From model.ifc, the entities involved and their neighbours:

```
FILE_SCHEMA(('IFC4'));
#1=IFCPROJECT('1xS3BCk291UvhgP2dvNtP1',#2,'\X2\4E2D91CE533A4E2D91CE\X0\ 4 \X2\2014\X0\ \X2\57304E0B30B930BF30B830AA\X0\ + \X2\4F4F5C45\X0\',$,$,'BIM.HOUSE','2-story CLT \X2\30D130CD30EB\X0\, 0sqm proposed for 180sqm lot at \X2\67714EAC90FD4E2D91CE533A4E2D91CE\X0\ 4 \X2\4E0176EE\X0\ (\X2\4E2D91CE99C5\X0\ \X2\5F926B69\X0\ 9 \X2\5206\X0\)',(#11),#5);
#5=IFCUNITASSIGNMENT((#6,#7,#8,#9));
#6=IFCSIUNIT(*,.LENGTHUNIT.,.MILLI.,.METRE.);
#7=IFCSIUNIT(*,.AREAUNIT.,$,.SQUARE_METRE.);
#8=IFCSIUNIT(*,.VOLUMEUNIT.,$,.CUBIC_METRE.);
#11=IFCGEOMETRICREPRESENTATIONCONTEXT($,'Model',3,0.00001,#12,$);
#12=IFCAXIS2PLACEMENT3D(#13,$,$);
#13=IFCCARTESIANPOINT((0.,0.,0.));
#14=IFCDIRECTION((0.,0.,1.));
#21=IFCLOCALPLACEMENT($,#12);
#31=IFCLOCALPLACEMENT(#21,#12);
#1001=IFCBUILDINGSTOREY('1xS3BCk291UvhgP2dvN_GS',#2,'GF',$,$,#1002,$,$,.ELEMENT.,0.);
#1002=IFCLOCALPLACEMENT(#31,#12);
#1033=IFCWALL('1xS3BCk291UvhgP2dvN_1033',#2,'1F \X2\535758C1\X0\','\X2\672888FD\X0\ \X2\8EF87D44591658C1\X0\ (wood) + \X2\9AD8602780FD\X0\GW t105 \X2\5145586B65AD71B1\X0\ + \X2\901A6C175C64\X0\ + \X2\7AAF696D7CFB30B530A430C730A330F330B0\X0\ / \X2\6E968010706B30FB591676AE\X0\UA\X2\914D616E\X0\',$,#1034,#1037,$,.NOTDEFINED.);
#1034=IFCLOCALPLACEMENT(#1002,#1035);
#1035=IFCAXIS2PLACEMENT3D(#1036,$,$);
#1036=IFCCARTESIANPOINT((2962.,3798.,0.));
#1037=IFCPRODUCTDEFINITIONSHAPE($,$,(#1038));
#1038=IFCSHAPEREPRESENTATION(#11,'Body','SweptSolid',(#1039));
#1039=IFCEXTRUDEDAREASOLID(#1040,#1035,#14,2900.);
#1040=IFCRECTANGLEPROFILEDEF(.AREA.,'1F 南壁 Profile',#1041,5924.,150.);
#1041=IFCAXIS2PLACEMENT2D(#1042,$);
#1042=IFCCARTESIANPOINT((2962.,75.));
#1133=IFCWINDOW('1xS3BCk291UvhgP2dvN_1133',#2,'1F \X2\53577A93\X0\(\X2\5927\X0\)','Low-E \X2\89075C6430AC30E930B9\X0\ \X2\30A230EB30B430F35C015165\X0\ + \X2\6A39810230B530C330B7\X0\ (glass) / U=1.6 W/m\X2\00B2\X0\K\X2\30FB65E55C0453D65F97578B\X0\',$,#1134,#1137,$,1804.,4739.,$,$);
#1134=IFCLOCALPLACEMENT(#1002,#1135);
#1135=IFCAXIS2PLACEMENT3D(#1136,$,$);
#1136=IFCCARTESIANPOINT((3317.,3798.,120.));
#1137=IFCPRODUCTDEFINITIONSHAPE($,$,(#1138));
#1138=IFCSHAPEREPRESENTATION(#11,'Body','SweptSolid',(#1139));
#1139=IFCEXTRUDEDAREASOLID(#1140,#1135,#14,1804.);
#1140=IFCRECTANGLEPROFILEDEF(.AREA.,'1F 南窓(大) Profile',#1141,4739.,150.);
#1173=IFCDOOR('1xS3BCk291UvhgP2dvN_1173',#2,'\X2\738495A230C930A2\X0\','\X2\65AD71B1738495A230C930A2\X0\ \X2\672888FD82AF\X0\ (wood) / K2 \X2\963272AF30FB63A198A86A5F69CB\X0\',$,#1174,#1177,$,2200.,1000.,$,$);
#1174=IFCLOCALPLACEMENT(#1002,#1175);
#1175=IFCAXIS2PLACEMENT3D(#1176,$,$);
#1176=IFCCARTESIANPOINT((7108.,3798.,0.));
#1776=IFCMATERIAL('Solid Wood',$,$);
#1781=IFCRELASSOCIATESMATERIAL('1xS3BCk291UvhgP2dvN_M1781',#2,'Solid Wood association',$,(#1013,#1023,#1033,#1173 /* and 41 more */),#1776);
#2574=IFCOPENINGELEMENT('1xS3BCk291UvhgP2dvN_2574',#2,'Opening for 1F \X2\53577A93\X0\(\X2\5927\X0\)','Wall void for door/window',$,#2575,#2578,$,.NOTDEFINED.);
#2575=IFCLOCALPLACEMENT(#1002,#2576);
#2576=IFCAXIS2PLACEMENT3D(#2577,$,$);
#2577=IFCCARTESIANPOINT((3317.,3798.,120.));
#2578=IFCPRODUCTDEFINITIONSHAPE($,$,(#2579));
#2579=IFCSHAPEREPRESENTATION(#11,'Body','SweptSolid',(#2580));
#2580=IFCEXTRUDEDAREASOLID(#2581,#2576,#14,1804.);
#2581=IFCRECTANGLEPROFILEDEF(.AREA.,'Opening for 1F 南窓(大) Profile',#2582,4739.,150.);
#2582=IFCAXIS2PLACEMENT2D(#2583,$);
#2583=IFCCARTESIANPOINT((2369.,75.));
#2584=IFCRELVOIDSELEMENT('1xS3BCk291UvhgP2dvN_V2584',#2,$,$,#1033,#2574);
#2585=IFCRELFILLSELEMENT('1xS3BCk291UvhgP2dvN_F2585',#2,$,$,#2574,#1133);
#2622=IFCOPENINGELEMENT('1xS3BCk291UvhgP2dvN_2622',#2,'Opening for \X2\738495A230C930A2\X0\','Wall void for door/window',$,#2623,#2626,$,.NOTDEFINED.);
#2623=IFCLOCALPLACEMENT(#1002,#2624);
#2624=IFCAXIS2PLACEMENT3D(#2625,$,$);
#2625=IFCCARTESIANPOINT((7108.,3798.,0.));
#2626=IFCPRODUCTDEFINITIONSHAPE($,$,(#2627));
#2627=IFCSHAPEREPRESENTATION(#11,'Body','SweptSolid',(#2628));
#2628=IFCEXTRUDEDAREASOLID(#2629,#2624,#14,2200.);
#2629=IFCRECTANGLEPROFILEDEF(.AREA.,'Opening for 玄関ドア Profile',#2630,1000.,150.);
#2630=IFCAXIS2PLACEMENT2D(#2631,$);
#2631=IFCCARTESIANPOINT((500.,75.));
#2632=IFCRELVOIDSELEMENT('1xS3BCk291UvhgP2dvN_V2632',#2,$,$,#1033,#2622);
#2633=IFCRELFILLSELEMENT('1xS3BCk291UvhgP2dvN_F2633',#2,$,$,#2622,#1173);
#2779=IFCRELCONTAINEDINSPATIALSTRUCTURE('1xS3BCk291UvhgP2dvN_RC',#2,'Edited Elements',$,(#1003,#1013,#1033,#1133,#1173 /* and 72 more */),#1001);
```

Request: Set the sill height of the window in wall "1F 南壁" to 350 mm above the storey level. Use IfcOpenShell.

```python
import numpy as np
import ifcopenshell
import ifcopenshell.api.geometry
import ifcopenshell.geom
import ifcopenshell.util.element
import ifcopenshell.util.placement
import ifcopenshell.util.shape
import ifcopenshell.util.unit

model = ifcopenshell.open("model.ifc")
unit_scale = ifcopenshell.util.unit.calculate_unit_scale(model)

window = model.by_guid("1xS3BCk291UvhgP2dvN_1133")
opening = window.FillsVoids[0].RelatingOpeningElement
storey = ifcopenshell.util.element.get_container(window, ifc_class="IfcBuildingStorey")
level = ifcopenshell.util.placement.get_local_placement(storey.ObjectPlacement)[2, 3]

# The opening's origin need not be at the sill, so measure its lowest point.
shape = ifcopenshell.geom.create_shape(ifcopenshell.geom.settings(), opening)
bottom = ifcopenshell.util.shape.get_shape_bottom_elevation(shape, shape.geometry) / unit_scale
dz = level + 0.35 / unit_scale - bottom

shift = np.array([0.0, 0.0, dz])
# The window is not placed relative to its opening, so move both.
for product in (opening, window):
    matrix = ifcopenshell.util.placement.get_local_placement(product.ObjectPlacement)
    matrix[:3, 3] += shift
    ifcopenshell.api.geometry.edit_object_placement(model, product=product, matrix=matrix, is_si=False)

print(f"moved by {dz * unit_scale:+.3f} m")

model.write("model_updated.ifc")
```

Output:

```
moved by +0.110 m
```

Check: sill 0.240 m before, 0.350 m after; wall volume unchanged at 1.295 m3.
